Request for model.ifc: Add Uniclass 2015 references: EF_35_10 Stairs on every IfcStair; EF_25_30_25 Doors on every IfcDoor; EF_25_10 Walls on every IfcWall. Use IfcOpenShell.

First a look at what the model holds.

```python
import ifcopenshell

model = ifcopenshell.open("model.ifc")
print(model.schema)
print("classifications:", [c.Name for c in model.by_type("IfcClassification")])
for ifc_class in ("IfcDoor", "IfcRoof", "IfcStair", "IfcWall", "IfcWindow"):
    print(ifc_class, len(model.by_type(ifc_class)))
```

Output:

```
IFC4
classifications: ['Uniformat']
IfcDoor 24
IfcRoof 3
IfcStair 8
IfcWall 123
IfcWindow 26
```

```python
import ifcopenshell
import ifcopenshell.api.classification

model = ifcopenshell.open("model.ifc")

system = ifcopenshell.api.classification.add_classification(model, classification="Uniclass 2015")

codes = {
    "IfcStair": ("EF_35_10", "Stairs"),
    "IfcDoor": ("EF_25_30_25", "Doors"),
    "IfcWall": ("EF_25_10", "Walls"),
}
for ifc_class, (code, name) in codes.items():
    products = model.by_type(ifc_class)
    ifcopenshell.api.classification.add_reference(
        model, products=products, classification=system, identification=code, name=name
    )
    print(code, len(products))

model.write("model_v2.ifc")
```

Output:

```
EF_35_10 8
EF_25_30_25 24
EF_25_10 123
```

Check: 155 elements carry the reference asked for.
